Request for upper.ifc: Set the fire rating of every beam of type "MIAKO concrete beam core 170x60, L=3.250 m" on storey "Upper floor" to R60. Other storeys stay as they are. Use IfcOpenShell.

First a look at what the model holds.

```python
import ifcopenshell
import ifcopenshell.util.element

model = ifcopenshell.open("upper.ifc")
print(model.schema)
storey = next(s for s in model.by_type("IfcBuildingStorey") if s.Name == "Upper floor")
beams = [e for e in ifcopenshell.util.element.get_decomposition(storey) if e.is_a("IfcBeam")]
seen = {}
for e in beams:
    element_type = ifcopenshell.util.element.get_type(e)
    key = (element_type.Name if element_type != e and element_type else None, ifcopenshell.util.element.get_pset(e, "Pset_BeamCommon", "FireRating"))
    seen[key] = seen.get(key, 0) + 1
for (name, value), count in sorted(seen.items(), key=str):
    print(count, "x", name, "|", value)
```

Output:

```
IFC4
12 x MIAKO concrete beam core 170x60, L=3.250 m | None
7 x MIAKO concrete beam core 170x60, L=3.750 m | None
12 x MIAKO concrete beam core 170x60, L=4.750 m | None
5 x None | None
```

```python
import ifcopenshell
import ifcopenshell.api.pset
import ifcopenshell.util.element

model = ifcopenshell.open("upper.ifc")

storey = next(s for s in model.by_type("IfcBuildingStorey") if s.Name == "Upper floor")
beams = [e for e in ifcopenshell.util.element.get_decomposition(storey) if e.is_a("IfcBeam")]

count = 0
for e in beams:
    element_type = ifcopenshell.util.element.get_type(e)
    if element_type in (None, e) or element_type.Name != "MIAKO concrete beam core 170x60, L=3.250 m":
        continue
    # add_pset returns the element's existing set when there is one.
    pset = ifcopenshell.api.pset.add_pset(model, product=e, name="Pset_BeamCommon")
    ifcopenshell.api.pset.edit_pset(model, pset=pset, properties={"FireRating": "R60"})
    count += 1

print(count, "beams updated")

model.write("upper_edited.ifc")
```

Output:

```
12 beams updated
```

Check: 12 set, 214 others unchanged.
